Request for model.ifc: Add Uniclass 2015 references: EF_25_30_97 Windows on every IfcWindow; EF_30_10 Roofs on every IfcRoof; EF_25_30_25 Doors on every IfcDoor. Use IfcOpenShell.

First a look at what the model holds.

```python
import ifcopenshell

model = ifcopenshell.open("model.ifc")
print(model.schema)
print("classifications:", [c.Name for c in model.by_type("IfcClassification")])
for ifc_class in ("IfcDoor", "IfcRoof", "IfcStair", "IfcWall", "IfcWindow"):
    print(ifc_class, len(model.by_type(ifc_class)))
```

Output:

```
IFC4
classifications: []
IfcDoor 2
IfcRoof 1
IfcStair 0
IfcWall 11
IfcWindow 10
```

```python
import ifcopenshell
import ifcopenshell.api.classification

model = ifcopenshell.open("model.ifc")

system = ifcopenshell.api.classification.add_classification(model, classification="Uniclass 2015")

codes = {
    "IfcWindow": ("EF_25_30_97", "Windows"),
    "IfcRoof": ("EF_30_10", "Roofs"),
    "IfcDoor": ("EF_25_30_25", "Doors"),
}
for ifc_class, (code, name) in codes.items():
    products = model.by_type(ifc_class)
    ifcopenshell.api.classification.add_reference(
        model, products=products, classification=system, identification=code, name=name
    )
    print(code, len(products))

model.write("model_v2.ifc")
```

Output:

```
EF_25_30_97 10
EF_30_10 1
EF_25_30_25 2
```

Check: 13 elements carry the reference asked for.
